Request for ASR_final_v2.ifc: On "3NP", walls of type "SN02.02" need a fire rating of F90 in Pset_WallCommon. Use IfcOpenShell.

First a look at what the model holds.

```python
import ifcopenshell
import ifcopenshell.util.element

model = ifcopenshell.open("ASR_final_v2.ifc")
print(model.schema)
storey = next(s for s in model.by_type("IfcBuildingStorey") if s.Name == "3NP")
walls = [e for e in ifcopenshell.util.element.get_decomposition(storey) if e.is_a("IfcWall")]
seen = {}
for e in walls:
    element_type = ifcopenshell.util.element.get_type(e)
    key = (element_type.Name if element_type != e and element_type else None, ifcopenshell.util.element.get_pset(e, "Pset_WallCommon", "FireRating"))
    seen[key] = seen.get(key, 0) + 1
for (name, value), count in sorted(seen.items(), key=str):
    print(count, "x", name, "|", value)
```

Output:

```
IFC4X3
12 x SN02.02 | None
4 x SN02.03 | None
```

```python
import ifcopenshell
import ifcopenshell.api.pset
import ifcopenshell.util.element

model = ifcopenshell.open("ASR_final_v2.ifc")

storey = next(s for s in model.by_type("IfcBuildingStorey") if s.Name == "3NP")
walls = [e for e in ifcopenshell.util.element.get_decomposition(storey) if e.is_a("IfcWall")]

count = 0
for e in walls:
    element_type = ifcopenshell.util.element.get_type(e)
    if element_type in (None, e) or element_type.Name != "SN02.02":
        continue
    # add_pset returns the element's existing set when there is one.
    pset = ifcopenshell.api.pset.add_pset(model, product=e, name="Pset_WallCommon")
    ifcopenshell.api.pset.edit_pset(model, pset=pset, properties={"FireRating": "F90"})
    count += 1

print(count, "walls updated")

model.write("ASR_final_v2_edited.ifc")
```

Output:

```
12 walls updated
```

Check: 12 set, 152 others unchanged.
